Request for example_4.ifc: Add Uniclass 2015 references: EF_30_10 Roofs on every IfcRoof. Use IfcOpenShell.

First a look at what the model holds.

```python
import ifcopenshell

model = ifcopenshell.open("example_4.ifc")
print(model.schema)
print("classifications:", [c.Name for c in model.by_type("IfcClassification")])
for ifc_class in ("IfcDoor", "IfcRoof", "IfcStair", "IfcWall", "IfcWindow"):
    print(ifc_class, len(model.by_type(ifc_class)))
```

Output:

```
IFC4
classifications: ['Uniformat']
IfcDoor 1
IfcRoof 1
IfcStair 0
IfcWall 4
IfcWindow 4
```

```python
import ifcopenshell
import ifcopenshell.api.classification

model = ifcopenshell.open("example_4.ifc")

system = ifcopenshell.api.classification.add_classification(model, classification="Uniclass 2015")

codes = {
    "IfcRoof": ("EF_30_10", "Roofs"),
}
for ifc_class, (code, name) in codes.items():
    products = model.by_type(ifc_class)
    ifcopenshell.api.classification.add_reference(
        model, products=products, classification=system, identification=code, name=name
    )
    print(code, len(products))

model.write("example_4_rev.ifc")
```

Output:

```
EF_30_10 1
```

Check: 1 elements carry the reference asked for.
